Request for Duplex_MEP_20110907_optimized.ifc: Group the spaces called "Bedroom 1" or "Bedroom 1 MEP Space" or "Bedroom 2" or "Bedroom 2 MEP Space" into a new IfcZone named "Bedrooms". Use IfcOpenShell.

First a look at what the model holds.

```python
import ifcopenshell

model = ifcopenshell.open("Duplex_MEP_20110907_optimized.ifc")
print(model.schema)
seen = {}
for space in model.by_type("IfcSpace"):
    seen[space.LongName] = seen.get(space.LongName, 0) + 1
for name, count in sorted(seen.items(), key=str):
    print(count, "x", name)
print("zones:", [z.Name for z in model.by_type("IfcZone")][:20])
```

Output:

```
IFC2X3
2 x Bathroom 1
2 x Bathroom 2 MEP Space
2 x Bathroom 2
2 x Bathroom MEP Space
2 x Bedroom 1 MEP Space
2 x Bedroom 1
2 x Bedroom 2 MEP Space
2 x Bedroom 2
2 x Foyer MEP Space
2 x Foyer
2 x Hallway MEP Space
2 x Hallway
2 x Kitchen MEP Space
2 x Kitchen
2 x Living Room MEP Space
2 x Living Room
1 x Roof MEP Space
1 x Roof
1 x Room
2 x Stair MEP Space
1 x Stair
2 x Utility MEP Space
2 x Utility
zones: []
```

```python
import ifcopenshell
import ifcopenshell.api.group
import ifcopenshell.api.root

model = ifcopenshell.open("Duplex_MEP_20110907_optimized.ifc")

names = {"Bedroom 1", "Bedroom 1 MEP Space", "Bedroom 2", "Bedroom 2 MEP Space"}
spaces = [s for s in model.by_type("IfcSpace") if s.LongName in names]

zone = ifcopenshell.api.root.create_entity(model, ifc_class="IfcZone", name="Bedrooms")
ifcopenshell.api.group.assign_group(model, products=spaces, group=zone)
print(len(spaces), "spaces in", zone.Name)

model.write("Duplex_MEP_20110907_optimized_edited.ifc")
```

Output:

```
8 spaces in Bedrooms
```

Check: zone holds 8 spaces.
